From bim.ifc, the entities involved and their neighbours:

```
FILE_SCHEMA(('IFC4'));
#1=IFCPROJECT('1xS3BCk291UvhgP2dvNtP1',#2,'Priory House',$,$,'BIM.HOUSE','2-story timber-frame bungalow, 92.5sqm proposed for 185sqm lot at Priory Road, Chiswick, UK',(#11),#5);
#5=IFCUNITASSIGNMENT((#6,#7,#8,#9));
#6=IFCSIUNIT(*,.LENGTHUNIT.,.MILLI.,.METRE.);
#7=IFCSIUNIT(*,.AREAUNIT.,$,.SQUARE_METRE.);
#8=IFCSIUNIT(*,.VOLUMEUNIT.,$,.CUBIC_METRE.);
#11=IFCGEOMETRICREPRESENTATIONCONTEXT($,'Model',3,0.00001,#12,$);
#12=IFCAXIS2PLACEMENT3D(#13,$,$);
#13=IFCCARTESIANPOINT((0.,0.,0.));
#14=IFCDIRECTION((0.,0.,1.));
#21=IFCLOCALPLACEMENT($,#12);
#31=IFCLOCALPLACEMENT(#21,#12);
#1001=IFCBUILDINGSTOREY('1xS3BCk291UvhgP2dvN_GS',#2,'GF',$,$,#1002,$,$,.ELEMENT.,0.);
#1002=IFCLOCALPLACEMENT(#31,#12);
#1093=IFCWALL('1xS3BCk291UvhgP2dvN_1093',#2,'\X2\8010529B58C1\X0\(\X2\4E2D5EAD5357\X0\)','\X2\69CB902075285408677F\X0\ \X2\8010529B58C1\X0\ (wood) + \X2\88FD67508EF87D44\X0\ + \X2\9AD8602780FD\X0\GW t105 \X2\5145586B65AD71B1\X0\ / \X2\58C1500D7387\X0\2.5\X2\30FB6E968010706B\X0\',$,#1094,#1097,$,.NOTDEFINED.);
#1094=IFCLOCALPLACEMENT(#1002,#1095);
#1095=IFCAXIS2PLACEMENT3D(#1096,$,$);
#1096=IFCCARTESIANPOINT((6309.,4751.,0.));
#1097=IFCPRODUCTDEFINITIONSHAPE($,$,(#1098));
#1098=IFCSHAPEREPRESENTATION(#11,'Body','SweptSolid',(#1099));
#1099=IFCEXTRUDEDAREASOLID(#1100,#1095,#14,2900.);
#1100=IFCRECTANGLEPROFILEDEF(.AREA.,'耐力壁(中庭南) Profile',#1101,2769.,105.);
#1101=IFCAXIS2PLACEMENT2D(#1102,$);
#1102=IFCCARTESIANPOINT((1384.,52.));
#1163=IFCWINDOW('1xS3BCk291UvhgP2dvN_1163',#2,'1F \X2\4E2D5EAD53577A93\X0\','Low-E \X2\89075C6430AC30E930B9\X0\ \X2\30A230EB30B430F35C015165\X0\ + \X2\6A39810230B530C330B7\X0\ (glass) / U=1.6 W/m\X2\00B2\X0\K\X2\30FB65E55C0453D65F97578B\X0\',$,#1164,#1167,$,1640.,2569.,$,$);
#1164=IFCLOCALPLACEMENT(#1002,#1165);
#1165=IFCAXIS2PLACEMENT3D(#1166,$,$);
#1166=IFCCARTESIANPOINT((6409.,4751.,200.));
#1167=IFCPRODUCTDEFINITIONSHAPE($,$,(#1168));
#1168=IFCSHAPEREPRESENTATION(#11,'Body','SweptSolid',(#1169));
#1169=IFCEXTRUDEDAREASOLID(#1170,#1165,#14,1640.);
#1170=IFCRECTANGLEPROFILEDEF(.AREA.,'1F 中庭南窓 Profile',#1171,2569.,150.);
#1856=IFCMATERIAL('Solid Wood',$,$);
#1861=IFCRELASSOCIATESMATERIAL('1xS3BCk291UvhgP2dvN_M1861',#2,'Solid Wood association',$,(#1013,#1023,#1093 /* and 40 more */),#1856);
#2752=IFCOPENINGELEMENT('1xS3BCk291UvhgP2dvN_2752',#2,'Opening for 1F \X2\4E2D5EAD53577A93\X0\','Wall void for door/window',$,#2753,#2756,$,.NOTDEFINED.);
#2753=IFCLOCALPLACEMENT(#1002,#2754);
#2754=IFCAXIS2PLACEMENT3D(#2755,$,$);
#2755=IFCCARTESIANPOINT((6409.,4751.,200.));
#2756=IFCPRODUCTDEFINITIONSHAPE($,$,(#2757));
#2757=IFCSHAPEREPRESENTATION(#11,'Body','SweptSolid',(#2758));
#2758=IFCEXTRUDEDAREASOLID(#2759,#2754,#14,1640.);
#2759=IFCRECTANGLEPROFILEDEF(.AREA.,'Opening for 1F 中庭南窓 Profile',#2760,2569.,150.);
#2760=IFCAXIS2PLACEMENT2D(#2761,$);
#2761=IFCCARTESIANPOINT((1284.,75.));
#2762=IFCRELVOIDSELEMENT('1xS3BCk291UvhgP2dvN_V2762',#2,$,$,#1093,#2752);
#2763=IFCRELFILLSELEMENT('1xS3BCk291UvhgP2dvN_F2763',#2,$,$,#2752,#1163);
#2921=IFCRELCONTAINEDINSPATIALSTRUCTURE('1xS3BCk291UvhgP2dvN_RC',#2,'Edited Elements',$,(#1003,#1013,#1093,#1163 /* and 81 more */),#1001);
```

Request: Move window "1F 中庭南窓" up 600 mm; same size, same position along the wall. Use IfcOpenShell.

```python
import numpy as np
import ifcopenshell
import ifcopenshell.api.geometry
import ifcopenshell.util.placement
import ifcopenshell.util.unit

model = ifcopenshell.open("bim.ifc")
unit_scale = ifcopenshell.util.unit.calculate_unit_scale(model)

window = model.by_id(1163)
opening = window.FillsVoids[0].RelatingOpeningElement
dz = 600.0

shift = np.array([0.0, 0.0, dz])
# The window is not placed relative to its opening, so move both.
for product in (opening, window):
    matrix = ifcopenshell.util.placement.get_local_placement(product.ObjectPlacement)
    matrix[:3, 3] += shift
    ifcopenshell.api.geometry.edit_object_placement(model, product=product, matrix=matrix, is_si=False)

print(f"moved by {dz * unit_scale:+.3f} m")

model.write("bim_edited.ifc")
```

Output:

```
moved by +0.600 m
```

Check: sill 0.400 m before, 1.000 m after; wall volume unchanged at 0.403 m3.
